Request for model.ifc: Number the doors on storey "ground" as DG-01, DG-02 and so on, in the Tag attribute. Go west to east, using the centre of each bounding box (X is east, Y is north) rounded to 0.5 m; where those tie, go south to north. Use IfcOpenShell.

First a look at what the model holds.

```python
import ifcopenshell
import ifcopenshell.util.element
import ifcopenshell.util.placement

model = ifcopenshell.open("model.ifc")
print(model.schema)
storey = next(s for s in model.by_type("IfcBuildingStorey") if s.Name == "ground")
doors = [e for e in ifcopenshell.util.element.get_decomposition(storey) if e.is_a("IfcDoor")]
for e in sorted(doors, key=lambda e: e.id()):
    origin = ifcopenshell.util.placement.get_local_placement(e.ObjectPlacement)[:3, 3]
    print(e.id(), e.Tag, e.Name, origin.round(2) + 0.0, sep=" | ")
```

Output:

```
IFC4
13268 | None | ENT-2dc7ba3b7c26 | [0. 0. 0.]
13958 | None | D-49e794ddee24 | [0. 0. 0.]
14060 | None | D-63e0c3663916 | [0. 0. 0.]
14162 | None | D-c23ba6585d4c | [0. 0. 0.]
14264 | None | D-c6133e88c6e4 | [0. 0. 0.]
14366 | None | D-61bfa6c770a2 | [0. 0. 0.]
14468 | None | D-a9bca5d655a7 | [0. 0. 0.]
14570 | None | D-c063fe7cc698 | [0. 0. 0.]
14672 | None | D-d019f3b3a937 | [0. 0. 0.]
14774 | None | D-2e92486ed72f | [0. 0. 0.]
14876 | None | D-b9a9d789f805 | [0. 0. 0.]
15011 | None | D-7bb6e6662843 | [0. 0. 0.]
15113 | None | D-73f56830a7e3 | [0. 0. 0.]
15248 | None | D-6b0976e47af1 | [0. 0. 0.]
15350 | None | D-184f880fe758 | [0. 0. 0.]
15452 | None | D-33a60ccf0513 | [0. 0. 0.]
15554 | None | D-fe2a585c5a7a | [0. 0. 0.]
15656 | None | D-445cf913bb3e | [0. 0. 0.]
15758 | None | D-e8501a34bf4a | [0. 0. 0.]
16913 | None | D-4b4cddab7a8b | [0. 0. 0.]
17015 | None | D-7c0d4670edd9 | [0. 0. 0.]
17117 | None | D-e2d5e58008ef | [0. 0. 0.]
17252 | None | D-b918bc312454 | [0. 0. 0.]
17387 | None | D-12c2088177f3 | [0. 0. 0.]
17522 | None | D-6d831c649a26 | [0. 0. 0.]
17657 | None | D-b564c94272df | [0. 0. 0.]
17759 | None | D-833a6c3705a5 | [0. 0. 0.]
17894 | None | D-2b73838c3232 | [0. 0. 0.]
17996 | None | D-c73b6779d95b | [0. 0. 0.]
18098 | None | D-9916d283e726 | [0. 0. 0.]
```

```python
import ifcopenshell
import ifcopenshell.geom
import ifcopenshell.util.element
import ifcopenshell.util.shape

model = ifcopenshell.open("model.ifc")
settings = ifcopenshell.geom.settings()
settings.set("use-world-coords", True)


def centre(element):
    shape = ifcopenshell.geom.create_shape(settings, element)
    return ifcopenshell.util.shape.get_bbox_centroid(shape.geometry)


storey = next(s for s in model.by_type("IfcBuildingStorey") if s.Name == "ground")
doors = [e for e in ifcopenshell.util.element.get_decomposition(storey) if e.is_a("IfcDoor")]

# Insertion points can sit at a corner or the storey origin, so sort by the geometry (in metres).
centres = {e: centre(e) for e in doors}
doors.sort(key=lambda e: (round(centres[e][0] / 0.5), centres[e][1]))

for i, e in enumerate(doors, start=1):
    number = f"DG-{i:02d}"
    e.Tag = number
    print(e.id(), number)

model.write("model-out.ifc")
```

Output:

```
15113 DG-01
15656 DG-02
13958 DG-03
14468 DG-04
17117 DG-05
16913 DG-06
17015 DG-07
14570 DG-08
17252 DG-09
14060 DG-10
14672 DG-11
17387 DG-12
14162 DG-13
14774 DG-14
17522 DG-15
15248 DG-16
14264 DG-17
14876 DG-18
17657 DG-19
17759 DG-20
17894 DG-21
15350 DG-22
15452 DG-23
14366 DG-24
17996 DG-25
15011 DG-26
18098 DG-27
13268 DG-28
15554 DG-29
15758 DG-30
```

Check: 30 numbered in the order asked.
